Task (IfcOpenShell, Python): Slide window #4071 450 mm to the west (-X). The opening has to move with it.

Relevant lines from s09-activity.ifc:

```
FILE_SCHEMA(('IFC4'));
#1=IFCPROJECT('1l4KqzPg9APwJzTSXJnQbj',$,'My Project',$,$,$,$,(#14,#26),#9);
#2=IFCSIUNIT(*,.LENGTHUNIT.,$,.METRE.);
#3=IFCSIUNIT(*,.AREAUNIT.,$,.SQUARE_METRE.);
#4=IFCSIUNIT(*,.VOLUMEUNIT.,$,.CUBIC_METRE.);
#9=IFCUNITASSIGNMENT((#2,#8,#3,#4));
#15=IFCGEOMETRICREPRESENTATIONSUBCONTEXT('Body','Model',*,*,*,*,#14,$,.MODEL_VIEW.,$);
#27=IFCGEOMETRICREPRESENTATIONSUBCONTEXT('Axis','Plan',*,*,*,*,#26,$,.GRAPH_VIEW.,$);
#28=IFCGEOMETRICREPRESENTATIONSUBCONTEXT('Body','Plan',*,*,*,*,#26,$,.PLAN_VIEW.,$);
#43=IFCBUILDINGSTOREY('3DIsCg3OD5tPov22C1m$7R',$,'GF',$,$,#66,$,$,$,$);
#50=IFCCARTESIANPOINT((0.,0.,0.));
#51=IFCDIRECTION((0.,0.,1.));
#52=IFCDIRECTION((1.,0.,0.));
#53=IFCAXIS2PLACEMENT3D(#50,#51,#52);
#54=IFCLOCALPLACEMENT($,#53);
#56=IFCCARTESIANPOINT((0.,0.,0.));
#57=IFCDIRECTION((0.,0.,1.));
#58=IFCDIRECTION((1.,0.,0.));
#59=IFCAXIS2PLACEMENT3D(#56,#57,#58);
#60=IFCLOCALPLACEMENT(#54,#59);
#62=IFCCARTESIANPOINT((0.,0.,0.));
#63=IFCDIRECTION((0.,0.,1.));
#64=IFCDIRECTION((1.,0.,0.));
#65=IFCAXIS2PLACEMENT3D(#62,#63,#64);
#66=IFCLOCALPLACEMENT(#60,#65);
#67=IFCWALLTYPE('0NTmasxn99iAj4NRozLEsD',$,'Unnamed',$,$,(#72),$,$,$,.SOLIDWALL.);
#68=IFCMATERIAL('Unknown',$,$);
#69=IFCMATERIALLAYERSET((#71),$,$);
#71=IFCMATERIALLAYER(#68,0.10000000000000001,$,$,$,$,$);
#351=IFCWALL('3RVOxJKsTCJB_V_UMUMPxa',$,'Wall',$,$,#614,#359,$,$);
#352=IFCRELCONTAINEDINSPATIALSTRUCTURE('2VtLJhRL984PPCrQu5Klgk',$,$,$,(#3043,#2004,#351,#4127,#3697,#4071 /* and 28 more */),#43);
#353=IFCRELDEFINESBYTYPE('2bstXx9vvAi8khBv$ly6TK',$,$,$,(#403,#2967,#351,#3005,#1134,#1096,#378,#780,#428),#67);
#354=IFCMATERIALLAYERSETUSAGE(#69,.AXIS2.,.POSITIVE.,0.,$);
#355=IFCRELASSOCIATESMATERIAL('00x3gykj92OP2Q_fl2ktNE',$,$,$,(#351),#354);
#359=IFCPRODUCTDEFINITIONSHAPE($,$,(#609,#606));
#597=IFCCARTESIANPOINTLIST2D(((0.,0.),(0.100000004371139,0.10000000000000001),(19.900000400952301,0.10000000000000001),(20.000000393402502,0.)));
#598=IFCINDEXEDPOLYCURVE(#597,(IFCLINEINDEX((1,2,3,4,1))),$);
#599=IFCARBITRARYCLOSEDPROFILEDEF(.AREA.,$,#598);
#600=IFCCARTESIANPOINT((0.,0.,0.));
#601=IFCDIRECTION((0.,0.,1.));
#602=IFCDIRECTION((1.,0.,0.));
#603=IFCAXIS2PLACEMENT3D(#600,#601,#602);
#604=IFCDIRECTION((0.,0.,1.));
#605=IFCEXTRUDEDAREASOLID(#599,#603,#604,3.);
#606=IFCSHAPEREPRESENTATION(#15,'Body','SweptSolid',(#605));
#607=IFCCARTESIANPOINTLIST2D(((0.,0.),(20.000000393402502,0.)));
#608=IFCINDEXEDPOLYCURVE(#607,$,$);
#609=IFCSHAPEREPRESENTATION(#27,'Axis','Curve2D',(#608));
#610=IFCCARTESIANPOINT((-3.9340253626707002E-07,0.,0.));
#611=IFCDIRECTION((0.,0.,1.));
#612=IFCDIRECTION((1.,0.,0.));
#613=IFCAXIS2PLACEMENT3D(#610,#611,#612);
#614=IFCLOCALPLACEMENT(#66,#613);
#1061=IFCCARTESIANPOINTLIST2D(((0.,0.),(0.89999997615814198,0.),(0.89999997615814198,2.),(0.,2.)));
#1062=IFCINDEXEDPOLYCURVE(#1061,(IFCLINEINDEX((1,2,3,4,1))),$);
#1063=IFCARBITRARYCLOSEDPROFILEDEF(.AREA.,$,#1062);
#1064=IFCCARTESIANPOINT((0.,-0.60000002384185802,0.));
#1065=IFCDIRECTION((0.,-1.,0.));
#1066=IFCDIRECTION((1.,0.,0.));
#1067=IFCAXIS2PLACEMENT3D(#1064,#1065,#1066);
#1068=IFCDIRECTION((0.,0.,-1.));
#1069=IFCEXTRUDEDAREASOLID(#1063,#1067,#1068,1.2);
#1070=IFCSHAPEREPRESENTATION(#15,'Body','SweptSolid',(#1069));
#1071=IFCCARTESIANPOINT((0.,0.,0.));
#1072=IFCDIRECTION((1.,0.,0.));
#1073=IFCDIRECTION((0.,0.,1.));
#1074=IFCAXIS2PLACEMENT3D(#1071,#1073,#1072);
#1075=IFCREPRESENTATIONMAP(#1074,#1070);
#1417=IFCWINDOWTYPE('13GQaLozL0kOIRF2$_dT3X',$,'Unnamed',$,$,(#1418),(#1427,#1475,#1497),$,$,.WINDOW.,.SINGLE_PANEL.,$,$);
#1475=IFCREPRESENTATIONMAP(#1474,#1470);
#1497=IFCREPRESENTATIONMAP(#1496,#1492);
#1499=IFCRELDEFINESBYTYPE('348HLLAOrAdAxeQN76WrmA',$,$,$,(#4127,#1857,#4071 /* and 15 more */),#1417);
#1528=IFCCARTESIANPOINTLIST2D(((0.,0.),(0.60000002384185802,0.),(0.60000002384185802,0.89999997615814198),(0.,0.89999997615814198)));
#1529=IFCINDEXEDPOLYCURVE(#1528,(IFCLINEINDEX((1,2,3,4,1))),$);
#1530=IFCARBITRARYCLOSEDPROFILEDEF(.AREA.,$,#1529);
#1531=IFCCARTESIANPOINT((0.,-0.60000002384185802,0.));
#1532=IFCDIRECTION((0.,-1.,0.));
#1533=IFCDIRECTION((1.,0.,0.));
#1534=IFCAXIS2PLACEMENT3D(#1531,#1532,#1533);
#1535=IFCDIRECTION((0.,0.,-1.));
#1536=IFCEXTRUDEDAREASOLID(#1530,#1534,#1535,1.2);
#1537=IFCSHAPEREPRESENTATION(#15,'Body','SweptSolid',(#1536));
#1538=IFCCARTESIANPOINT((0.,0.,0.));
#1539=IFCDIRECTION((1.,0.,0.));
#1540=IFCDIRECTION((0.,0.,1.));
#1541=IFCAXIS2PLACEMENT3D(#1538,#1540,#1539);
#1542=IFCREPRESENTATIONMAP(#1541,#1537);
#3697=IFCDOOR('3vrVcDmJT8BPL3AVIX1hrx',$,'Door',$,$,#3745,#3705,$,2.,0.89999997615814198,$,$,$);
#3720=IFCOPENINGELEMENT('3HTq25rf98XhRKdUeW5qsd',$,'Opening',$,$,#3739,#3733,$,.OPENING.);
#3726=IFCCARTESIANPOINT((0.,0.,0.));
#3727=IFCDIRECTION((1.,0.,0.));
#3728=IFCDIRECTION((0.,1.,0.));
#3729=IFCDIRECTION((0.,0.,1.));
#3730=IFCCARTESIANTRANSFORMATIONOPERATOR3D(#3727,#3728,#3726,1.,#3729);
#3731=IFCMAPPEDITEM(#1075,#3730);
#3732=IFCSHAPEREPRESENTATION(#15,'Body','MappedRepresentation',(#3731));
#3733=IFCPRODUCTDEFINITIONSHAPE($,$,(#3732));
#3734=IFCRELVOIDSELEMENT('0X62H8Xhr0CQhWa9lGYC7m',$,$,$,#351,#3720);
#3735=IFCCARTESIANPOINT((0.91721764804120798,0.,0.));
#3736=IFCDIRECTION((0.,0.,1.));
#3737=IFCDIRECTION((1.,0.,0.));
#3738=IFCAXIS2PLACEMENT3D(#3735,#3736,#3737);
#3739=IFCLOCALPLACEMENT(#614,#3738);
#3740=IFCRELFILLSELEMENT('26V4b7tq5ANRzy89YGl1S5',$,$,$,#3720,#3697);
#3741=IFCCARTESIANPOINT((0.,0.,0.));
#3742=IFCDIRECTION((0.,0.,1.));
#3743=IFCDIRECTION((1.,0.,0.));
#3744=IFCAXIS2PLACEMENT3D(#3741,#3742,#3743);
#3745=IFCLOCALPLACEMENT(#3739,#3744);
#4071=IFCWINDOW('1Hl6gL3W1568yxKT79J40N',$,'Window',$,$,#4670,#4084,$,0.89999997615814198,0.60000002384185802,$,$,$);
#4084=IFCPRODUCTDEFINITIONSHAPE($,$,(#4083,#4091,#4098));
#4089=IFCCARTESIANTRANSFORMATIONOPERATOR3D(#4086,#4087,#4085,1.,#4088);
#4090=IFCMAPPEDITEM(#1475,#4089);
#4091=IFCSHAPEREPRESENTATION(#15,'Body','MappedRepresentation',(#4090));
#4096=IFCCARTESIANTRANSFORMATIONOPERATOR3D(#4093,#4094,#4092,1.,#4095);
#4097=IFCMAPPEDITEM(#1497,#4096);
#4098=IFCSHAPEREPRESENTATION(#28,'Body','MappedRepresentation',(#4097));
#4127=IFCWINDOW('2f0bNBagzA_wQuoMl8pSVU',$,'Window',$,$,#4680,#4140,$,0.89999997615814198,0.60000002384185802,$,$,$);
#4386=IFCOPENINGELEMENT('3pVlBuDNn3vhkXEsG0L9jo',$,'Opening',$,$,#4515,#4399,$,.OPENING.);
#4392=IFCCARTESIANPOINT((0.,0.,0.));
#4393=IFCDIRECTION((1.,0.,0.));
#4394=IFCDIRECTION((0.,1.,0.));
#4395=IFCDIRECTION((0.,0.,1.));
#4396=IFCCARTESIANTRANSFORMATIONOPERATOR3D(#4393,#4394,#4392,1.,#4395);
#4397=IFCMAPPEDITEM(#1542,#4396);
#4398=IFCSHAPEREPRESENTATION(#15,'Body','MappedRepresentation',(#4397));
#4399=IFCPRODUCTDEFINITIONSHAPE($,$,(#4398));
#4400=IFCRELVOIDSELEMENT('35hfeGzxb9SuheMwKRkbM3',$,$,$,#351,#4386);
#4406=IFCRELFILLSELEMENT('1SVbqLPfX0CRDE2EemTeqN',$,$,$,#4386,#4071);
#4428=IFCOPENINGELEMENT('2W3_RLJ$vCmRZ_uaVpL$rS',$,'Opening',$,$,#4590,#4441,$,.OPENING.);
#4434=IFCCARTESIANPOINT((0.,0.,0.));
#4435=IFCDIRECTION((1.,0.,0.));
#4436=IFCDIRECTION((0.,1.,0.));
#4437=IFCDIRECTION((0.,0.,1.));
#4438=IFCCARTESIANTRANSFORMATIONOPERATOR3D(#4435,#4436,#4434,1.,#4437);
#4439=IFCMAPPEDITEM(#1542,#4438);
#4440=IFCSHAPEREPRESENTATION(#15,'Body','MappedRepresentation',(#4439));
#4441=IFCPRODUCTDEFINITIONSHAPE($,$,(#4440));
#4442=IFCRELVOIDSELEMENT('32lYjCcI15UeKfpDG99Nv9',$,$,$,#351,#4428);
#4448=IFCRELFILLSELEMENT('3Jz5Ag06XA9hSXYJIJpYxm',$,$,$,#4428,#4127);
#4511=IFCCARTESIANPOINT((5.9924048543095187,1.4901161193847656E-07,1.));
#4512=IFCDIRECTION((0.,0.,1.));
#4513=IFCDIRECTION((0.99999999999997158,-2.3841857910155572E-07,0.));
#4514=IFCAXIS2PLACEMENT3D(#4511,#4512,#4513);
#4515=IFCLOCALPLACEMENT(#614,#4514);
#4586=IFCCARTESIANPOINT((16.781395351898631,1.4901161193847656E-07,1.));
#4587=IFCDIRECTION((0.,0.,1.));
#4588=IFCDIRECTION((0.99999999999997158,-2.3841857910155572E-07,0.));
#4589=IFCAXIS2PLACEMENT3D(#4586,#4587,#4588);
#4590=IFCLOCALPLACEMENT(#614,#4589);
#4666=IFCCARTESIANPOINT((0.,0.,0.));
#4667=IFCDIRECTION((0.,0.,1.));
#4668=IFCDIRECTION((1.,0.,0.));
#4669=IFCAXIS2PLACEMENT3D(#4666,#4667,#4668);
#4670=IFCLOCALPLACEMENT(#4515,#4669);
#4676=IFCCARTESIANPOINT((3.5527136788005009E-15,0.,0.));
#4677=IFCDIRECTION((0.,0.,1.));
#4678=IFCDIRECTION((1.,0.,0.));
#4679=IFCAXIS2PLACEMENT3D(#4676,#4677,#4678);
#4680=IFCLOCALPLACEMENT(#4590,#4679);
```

```python
import ifcopenshell
import ifcopenshell.api.geometry
import ifcopenshell.util.placement
import ifcopenshell.util.unit

model = ifcopenshell.open("s09-activity.ifc")
unit_scale = ifcopenshell.util.unit.calculate_unit_scale(model)

window = model.by_guid("1Hl6gL3W1568yxKT79J40N")
opening = window.FillsVoids[0].RelatingOpeningElement
wall = opening.VoidsElements[0].RelatingBuildingElement

wall_matrix = ifcopenshell.util.placement.get_local_placement(wall.ObjectPlacement)
shift = wall_matrix[:3, 0] * -0.45 / unit_scale
before = ifcopenshell.util.placement.get_local_placement(window.ObjectPlacement)[:3, 3].copy()

# The window is placed relative to its opening, so it follows when the opening moves.
matrix = ifcopenshell.util.placement.get_local_placement(opening.ObjectPlacement)
matrix[:3, 3] += shift
ifcopenshell.api.geometry.edit_object_placement(
    model, product=opening, matrix=matrix, is_si=False, should_transform_children=True
)

after = ifcopenshell.util.placement.get_local_placement(window.ObjectPlacement)[:3, 3]
print("window moved by", (after - before).round(3) + 0.0)

model.write("s09-activity-out.ifc")
```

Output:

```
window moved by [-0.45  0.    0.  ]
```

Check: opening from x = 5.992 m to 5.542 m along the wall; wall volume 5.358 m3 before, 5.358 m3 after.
